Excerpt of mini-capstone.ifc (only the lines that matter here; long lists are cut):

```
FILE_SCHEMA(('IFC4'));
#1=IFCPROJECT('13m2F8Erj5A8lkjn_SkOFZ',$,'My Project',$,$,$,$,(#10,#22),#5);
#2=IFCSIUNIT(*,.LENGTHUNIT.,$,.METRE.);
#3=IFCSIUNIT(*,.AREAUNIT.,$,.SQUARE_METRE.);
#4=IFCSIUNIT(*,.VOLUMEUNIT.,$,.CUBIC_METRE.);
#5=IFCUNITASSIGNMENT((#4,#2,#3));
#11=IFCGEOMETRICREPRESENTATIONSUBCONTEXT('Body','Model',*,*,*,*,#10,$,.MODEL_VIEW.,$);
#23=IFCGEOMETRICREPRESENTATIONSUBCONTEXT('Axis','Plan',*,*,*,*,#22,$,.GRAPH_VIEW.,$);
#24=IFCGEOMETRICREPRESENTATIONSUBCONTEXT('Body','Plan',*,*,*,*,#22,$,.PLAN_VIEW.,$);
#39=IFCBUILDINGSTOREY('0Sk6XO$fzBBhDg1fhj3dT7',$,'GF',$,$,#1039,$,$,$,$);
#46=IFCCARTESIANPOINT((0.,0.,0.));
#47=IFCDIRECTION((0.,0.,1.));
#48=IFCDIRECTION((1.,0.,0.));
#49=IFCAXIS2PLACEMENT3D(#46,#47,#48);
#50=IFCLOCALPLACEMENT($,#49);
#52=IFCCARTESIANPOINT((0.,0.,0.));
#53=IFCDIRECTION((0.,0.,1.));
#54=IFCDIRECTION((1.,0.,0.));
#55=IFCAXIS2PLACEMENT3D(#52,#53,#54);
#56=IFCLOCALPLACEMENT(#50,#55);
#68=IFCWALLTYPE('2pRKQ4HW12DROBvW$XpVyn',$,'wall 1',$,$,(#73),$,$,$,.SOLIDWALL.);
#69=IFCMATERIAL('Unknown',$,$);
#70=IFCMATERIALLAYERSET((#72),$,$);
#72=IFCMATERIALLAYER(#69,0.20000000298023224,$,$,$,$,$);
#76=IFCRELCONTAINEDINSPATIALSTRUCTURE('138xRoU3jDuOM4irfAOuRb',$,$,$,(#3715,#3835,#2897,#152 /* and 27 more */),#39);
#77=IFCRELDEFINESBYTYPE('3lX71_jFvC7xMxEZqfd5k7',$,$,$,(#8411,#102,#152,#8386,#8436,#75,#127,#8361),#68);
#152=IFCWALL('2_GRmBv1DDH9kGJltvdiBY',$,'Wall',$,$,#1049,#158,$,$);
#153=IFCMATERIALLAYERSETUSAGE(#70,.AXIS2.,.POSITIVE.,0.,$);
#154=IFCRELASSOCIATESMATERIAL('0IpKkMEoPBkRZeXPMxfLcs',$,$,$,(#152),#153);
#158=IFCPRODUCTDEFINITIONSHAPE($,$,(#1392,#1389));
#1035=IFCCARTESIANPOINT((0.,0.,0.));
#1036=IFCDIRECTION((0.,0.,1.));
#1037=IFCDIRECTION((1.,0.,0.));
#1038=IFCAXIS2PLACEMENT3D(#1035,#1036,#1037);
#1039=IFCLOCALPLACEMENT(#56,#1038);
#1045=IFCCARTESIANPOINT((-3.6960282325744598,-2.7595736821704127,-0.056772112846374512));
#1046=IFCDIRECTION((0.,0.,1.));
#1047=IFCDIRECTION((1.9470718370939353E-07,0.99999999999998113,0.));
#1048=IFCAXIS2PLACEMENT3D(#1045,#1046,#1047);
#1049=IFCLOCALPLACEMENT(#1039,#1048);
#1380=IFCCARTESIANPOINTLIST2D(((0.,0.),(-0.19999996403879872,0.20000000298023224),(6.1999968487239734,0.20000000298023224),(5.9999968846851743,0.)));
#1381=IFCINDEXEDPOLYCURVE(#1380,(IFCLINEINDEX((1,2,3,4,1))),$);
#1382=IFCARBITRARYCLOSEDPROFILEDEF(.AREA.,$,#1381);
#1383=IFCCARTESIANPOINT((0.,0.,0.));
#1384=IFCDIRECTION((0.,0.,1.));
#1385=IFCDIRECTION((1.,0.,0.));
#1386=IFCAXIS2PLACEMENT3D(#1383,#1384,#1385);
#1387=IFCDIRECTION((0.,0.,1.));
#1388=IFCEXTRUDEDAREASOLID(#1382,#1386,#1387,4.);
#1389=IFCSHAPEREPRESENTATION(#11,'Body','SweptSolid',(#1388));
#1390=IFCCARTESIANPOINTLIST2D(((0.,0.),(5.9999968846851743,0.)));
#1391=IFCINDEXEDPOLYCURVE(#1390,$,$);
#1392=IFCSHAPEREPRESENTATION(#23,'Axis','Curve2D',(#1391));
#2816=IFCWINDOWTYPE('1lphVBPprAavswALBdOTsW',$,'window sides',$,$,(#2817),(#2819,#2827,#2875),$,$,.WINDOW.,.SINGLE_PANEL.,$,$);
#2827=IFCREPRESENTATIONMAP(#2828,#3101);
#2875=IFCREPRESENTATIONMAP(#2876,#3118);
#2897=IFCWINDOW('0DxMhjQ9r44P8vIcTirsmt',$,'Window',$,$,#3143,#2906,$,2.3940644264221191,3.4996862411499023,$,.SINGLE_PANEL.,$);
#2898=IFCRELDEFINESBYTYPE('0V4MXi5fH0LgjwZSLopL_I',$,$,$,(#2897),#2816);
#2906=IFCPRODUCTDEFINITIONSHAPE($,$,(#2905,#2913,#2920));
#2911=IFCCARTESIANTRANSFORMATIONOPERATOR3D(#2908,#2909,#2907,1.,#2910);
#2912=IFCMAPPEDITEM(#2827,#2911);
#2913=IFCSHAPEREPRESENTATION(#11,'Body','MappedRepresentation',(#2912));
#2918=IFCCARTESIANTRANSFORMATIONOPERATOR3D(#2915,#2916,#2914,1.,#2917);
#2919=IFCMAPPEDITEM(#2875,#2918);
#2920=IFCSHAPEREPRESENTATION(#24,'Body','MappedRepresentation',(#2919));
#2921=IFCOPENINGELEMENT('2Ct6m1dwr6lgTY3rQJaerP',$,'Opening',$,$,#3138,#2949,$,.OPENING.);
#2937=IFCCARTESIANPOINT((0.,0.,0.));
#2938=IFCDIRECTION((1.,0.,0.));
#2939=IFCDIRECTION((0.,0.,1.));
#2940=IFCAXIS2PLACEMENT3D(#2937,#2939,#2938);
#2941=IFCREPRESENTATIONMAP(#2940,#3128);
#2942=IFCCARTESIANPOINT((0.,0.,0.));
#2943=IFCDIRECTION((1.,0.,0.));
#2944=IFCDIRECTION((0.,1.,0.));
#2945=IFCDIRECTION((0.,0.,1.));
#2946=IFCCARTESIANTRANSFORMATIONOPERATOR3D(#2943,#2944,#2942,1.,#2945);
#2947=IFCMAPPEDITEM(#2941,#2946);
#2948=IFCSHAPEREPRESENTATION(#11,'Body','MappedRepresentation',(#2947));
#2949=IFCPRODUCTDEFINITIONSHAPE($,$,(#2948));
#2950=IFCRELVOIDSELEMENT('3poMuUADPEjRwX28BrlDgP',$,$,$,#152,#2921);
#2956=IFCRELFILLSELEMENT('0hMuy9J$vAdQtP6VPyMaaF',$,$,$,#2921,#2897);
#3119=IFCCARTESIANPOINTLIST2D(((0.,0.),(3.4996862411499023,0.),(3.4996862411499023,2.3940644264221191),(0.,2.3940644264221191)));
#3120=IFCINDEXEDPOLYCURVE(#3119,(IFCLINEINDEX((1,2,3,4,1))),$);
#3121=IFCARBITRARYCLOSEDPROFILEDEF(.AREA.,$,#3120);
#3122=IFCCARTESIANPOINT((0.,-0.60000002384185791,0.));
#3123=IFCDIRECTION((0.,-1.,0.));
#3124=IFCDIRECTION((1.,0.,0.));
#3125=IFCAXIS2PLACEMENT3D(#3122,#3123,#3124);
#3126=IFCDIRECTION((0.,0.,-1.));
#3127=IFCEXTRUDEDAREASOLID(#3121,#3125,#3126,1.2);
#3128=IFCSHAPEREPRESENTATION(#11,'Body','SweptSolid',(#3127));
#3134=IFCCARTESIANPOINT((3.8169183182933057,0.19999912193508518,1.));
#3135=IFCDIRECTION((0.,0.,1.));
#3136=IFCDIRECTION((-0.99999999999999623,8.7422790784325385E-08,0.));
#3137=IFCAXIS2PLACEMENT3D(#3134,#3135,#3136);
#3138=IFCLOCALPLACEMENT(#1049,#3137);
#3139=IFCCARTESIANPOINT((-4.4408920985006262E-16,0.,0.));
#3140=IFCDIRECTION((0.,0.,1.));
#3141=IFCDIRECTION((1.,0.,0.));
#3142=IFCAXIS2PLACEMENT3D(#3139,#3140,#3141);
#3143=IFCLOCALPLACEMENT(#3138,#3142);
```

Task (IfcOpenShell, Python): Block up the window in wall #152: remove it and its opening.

```python
import ifcopenshell
import ifcopenshell.api.feature
import ifcopenshell.api.root
import ifcopenshell.geom
import ifcopenshell.util.shape

model = ifcopenshell.open("mini-capstone.ifc")
settings = ifcopenshell.geom.settings()


def volume(element):
    """Net volume in cubic metres, openings subtracted."""
    shape = ifcopenshell.geom.create_shape(settings, element)
    return ifcopenshell.util.shape.get_volume(shape.geometry)


window = model.by_guid("0DxMhjQ9r44P8vIcTirsmt")
opening = window.FillsVoids[0].RelatingOpeningElement
wall = opening.VoidsElements[0].RelatingBuildingElement
before = volume(wall)

ifcopenshell.api.root.remove_product(model, product=window)
ifcopenshell.api.feature.remove_feature(model, feature=opening)

after = volume(wall)

print(f"wall volume {before:.3f} -> {after:.3f} m3")

model.write("mini-capstone_updated.ifc")
```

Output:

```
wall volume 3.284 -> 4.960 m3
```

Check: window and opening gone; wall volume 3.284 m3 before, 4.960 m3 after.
